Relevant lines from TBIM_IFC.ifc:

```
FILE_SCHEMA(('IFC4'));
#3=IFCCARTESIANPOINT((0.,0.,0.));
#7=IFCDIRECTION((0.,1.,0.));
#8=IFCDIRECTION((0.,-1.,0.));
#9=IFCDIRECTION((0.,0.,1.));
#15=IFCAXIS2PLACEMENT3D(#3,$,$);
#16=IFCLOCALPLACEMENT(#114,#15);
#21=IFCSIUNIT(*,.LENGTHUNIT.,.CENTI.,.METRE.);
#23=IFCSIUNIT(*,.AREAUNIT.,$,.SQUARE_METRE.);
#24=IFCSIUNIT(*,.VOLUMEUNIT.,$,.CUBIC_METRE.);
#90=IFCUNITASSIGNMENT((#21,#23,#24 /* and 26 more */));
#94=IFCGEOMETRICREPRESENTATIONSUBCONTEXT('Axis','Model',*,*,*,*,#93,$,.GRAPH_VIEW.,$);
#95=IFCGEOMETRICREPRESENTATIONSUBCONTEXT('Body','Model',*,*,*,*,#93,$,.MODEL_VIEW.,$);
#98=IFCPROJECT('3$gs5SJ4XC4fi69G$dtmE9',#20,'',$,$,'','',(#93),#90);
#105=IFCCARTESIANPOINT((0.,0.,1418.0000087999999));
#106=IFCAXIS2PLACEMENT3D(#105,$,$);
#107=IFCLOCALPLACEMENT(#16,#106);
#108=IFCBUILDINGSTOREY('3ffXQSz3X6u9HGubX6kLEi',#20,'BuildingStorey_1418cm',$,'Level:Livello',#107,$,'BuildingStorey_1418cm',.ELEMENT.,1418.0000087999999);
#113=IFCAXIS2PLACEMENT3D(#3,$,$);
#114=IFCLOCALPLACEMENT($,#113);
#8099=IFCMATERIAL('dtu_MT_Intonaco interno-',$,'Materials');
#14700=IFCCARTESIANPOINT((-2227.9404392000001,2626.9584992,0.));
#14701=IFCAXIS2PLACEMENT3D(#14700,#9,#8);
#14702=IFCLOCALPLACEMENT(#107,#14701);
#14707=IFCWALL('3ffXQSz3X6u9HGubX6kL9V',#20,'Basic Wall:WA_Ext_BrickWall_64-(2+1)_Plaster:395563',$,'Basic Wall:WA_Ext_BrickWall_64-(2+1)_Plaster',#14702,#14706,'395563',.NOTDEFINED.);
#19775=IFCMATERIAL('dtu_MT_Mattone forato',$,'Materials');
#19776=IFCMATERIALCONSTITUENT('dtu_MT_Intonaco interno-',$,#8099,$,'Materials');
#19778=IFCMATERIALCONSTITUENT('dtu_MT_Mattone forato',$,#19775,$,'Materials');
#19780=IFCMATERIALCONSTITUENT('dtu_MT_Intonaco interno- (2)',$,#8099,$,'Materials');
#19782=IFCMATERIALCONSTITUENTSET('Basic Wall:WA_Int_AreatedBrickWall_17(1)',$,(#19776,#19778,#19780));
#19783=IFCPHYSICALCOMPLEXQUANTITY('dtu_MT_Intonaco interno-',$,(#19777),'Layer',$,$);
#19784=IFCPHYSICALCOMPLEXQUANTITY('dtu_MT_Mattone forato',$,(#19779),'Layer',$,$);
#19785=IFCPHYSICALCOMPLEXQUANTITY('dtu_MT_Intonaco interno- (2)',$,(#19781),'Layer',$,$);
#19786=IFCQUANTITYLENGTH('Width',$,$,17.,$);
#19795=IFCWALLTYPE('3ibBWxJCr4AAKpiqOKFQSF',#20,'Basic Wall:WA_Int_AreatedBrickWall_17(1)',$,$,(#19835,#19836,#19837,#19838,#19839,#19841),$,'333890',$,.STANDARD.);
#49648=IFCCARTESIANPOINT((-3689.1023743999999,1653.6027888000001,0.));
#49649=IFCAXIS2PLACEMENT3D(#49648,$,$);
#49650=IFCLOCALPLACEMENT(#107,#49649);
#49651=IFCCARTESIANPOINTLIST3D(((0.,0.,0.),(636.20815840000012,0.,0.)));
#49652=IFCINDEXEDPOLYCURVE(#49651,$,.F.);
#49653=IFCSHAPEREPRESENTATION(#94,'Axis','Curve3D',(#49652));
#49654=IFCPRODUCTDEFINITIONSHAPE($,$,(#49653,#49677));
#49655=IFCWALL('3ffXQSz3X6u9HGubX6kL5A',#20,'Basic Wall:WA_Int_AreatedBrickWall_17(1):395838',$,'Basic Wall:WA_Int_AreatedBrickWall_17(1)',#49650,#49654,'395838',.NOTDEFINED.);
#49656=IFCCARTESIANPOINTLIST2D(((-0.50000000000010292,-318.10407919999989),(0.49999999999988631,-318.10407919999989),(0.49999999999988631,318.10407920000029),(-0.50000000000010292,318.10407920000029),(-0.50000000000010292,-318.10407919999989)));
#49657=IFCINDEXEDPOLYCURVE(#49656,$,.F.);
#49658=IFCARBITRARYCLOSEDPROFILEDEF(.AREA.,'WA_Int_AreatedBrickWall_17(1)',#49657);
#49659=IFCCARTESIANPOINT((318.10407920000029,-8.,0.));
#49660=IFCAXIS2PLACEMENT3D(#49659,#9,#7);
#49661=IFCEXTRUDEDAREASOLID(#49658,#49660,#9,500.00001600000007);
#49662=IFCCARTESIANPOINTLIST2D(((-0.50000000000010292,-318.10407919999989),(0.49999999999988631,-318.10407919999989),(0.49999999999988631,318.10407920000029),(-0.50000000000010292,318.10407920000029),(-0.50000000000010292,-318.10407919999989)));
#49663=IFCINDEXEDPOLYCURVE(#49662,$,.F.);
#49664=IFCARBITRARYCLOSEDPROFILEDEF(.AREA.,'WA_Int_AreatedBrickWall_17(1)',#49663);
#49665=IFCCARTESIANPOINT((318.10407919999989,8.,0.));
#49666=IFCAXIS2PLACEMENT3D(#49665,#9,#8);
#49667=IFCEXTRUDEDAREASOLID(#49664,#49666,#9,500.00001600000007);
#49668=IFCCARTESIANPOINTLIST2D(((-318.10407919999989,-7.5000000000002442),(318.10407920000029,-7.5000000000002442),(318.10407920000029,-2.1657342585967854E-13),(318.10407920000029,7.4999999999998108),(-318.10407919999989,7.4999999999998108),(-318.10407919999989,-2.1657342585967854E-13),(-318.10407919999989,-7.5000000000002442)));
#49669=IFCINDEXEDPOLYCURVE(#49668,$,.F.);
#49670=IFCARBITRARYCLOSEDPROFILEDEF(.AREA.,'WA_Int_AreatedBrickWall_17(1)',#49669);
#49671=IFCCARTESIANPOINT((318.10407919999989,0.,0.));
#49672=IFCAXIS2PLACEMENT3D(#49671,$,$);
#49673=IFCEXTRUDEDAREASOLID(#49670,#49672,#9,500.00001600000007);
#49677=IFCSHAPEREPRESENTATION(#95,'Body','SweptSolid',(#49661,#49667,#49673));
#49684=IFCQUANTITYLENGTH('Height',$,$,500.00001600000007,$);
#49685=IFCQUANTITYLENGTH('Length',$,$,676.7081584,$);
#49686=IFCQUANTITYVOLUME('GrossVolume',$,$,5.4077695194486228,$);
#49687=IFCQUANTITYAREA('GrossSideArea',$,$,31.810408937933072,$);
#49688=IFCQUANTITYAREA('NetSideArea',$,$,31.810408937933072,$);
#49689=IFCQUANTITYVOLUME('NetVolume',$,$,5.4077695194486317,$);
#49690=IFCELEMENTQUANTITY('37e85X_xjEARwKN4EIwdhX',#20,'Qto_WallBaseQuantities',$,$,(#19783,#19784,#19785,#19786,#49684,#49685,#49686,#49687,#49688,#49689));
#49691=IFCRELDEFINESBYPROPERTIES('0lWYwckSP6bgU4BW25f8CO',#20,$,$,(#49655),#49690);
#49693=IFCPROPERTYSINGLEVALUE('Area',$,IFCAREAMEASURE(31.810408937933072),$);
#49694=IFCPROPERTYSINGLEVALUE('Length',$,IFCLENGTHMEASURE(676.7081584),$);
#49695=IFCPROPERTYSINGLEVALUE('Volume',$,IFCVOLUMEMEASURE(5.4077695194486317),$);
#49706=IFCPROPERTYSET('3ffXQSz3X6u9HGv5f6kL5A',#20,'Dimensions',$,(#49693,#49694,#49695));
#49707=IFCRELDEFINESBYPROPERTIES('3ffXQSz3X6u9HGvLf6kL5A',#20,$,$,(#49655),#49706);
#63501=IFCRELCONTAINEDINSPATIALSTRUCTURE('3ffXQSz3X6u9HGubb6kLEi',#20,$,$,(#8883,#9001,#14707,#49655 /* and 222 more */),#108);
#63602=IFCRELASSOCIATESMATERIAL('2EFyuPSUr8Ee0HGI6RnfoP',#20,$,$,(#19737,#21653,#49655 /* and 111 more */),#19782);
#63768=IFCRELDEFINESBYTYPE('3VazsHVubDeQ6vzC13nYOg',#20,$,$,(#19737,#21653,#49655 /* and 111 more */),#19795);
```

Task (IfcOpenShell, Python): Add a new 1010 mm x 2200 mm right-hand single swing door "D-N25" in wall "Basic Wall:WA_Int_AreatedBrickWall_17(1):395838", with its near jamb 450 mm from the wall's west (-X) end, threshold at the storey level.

```python
import numpy as np
import ifcopenshell
import ifcopenshell.api.feature
import ifcopenshell.api.geometry
import ifcopenshell.api.pset
import ifcopenshell.api.root
import ifcopenshell.api.spatial
import ifcopenshell.geom
import ifcopenshell.util.element
import ifcopenshell.util.placement
import ifcopenshell.util.representation
import ifcopenshell.util.shape
import ifcopenshell.util.unit

model = ifcopenshell.open("TBIM_IFC.ifc")
unit_scale = ifcopenshell.util.unit.calculate_unit_scale(model)
area_scale = ifcopenshell.util.unit.calculate_unit_scale(model, "AREAUNIT")
volume_scale = ifcopenshell.util.unit.calculate_unit_scale(model, "VOLUMEUNIT")
settings = ifcopenshell.geom.settings()


def volume(element):
    """Net volume in cubic metres, openings subtracted."""
    shape = ifcopenshell.geom.create_shape(settings, element)
    return ifcopenshell.util.shape.get_volume(shape.geometry)


wall = model.by_guid("3ffXQSz3X6u9HGubX6kL5A")
storey = ifcopenshell.util.element.get_container(wall, ifc_class="IfcBuildingStorey")
context = ifcopenshell.util.representation.get_context(model, "Model", "Body", "MODEL_VIEW")
before = volume(wall)

width, height, from_end, sill = 1.01, 2.2, 0.45, 0.0  # metres

# The wall runs along its own X axis, and the end named is its -X end.
wall_shape = ifcopenshell.geom.create_shape(settings, wall)
x, y, z = ifcopenshell.util.shape.get_vertices(wall_shape.geometry).T
start = x.min() + from_end
face, thickness = float(y.min()), float(y.max() - y.min())
wall_matrix = ifcopenshell.util.placement.get_local_placement(wall.ObjectPlacement)
level = ifcopenshell.util.placement.get_local_placement(storey.ObjectPlacement)[2, 3]


def in_wall(x, y):
    """Placement at x, y metres in the wall's axes, at sill height."""
    matrix = wall_matrix.copy()
    matrix[:, 3] = wall_matrix @ np.array([x / unit_scale, y / unit_scale, 0.0, 1.0])
    matrix[2, 3] = level + sill / unit_scale
    return matrix


# Opening: a box that overshoots both wall faces by 50 mm.
opening = ifcopenshell.api.root.create_entity(model, ifc_class="IfcOpeningElement", predefined_type="OPENING")
box = ifcopenshell.api.geometry.add_wall_representation(
    model, context=context, length=width, height=height, thickness=thickness + 0.1
)
ifcopenshell.api.geometry.assign_representation(model, product=opening, representation=box)
ifcopenshell.api.geometry.edit_object_placement(model, product=opening, matrix=in_wall(start, face - 0.05), is_si=False)
ifcopenshell.api.feature.add_feature(model, feature=opening, element=wall)

door = ifcopenshell.api.root.create_entity(model, ifc_class="IfcDoor", name="D-N25", predefined_type="DOOR")
door.OverallWidth, door.OverallHeight = width / unit_scale, height / unit_scale
door.OperationType = "SINGLE_SWING_RIGHT"
body = ifcopenshell.api.geometry.add_door_representation(
    model,
    context=context,
    overall_width=door.OverallWidth,
    overall_height=door.OverallHeight,
    operation_type="SINGLE_SWING_RIGHT",
    lining_properties={"LiningDepth": thickness / unit_scale, "ThresholdDepth": thickness / unit_scale},
)
ifcopenshell.api.geometry.assign_representation(model, product=door, representation=body)
ifcopenshell.api.spatial.assign_container(model, products=[door], relating_structure=storey)
ifcopenshell.api.feature.add_filling(model, opening=opening, element=door)

# The lining spans the wall, so the door starts at the wall face.
ifcopenshell.api.geometry.edit_object_placement(model, product=door, matrix=in_wall(start, face), is_si=False)

after = volume(wall)

# Update the wall's stored quantities.
qto = model.by_id(ifcopenshell.util.element.get_pset(wall, "Qto_WallBaseQuantities", should_inherit=False)["id"])
ifcopenshell.api.pset.edit_qto(model, qto=qto, properties={
    "NetSideArea": after / thickness / area_scale,
    "NetVolume": after / volume_scale,
})
pset = model.by_id(ifcopenshell.util.element.get_pset(wall, "Dimensions", should_inherit=False)["id"])
ifcopenshell.api.pset.edit_pset(model, pset=pset, properties={
    "Area": model.create_entity("IfcAreaMeasure", after / thickness / area_scale),
    "Volume": model.create_entity("IfcVolumeMeasure", after / volume_scale),
})

print(f"wall volume {before:.3f} -> {after:.3f} m3")

model.write("TBIM_IFC_v2.ifc")
```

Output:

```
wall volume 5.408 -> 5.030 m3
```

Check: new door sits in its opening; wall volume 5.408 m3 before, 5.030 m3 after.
